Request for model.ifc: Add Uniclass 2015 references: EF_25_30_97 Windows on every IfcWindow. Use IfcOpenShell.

First a look at what the model holds.

```python
import ifcopenshell

model = ifcopenshell.open("model.ifc")
print(model.schema)
print("classifications:", [c.Name for c in model.by_type("IfcClassification")])
for ifc_class in ("IfcDoor", "IfcRoof", "IfcStair", "IfcWall", "IfcWindow"):
    print(ifc_class, len(model.by_type(ifc_class)))
```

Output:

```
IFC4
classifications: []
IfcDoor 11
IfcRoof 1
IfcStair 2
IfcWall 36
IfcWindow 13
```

```python
import ifcopenshell
import ifcopenshell.api.classification

model = ifcopenshell.open("model.ifc")

system = ifcopenshell.api.classification.add_classification(model, classification="Uniclass 2015")

codes = {
    "IfcWindow": ("EF_25_30_97", "Windows"),
}
for ifc_class, (code, name) in codes.items():
    products = model.by_type(ifc_class)
    ifcopenshell.api.classification.add_reference(
        model, products=products, classification=system, identification=code, name=name
    )
    print(code, len(products))

model.write("model_v2.ifc")
```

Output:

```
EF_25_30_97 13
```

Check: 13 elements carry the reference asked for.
